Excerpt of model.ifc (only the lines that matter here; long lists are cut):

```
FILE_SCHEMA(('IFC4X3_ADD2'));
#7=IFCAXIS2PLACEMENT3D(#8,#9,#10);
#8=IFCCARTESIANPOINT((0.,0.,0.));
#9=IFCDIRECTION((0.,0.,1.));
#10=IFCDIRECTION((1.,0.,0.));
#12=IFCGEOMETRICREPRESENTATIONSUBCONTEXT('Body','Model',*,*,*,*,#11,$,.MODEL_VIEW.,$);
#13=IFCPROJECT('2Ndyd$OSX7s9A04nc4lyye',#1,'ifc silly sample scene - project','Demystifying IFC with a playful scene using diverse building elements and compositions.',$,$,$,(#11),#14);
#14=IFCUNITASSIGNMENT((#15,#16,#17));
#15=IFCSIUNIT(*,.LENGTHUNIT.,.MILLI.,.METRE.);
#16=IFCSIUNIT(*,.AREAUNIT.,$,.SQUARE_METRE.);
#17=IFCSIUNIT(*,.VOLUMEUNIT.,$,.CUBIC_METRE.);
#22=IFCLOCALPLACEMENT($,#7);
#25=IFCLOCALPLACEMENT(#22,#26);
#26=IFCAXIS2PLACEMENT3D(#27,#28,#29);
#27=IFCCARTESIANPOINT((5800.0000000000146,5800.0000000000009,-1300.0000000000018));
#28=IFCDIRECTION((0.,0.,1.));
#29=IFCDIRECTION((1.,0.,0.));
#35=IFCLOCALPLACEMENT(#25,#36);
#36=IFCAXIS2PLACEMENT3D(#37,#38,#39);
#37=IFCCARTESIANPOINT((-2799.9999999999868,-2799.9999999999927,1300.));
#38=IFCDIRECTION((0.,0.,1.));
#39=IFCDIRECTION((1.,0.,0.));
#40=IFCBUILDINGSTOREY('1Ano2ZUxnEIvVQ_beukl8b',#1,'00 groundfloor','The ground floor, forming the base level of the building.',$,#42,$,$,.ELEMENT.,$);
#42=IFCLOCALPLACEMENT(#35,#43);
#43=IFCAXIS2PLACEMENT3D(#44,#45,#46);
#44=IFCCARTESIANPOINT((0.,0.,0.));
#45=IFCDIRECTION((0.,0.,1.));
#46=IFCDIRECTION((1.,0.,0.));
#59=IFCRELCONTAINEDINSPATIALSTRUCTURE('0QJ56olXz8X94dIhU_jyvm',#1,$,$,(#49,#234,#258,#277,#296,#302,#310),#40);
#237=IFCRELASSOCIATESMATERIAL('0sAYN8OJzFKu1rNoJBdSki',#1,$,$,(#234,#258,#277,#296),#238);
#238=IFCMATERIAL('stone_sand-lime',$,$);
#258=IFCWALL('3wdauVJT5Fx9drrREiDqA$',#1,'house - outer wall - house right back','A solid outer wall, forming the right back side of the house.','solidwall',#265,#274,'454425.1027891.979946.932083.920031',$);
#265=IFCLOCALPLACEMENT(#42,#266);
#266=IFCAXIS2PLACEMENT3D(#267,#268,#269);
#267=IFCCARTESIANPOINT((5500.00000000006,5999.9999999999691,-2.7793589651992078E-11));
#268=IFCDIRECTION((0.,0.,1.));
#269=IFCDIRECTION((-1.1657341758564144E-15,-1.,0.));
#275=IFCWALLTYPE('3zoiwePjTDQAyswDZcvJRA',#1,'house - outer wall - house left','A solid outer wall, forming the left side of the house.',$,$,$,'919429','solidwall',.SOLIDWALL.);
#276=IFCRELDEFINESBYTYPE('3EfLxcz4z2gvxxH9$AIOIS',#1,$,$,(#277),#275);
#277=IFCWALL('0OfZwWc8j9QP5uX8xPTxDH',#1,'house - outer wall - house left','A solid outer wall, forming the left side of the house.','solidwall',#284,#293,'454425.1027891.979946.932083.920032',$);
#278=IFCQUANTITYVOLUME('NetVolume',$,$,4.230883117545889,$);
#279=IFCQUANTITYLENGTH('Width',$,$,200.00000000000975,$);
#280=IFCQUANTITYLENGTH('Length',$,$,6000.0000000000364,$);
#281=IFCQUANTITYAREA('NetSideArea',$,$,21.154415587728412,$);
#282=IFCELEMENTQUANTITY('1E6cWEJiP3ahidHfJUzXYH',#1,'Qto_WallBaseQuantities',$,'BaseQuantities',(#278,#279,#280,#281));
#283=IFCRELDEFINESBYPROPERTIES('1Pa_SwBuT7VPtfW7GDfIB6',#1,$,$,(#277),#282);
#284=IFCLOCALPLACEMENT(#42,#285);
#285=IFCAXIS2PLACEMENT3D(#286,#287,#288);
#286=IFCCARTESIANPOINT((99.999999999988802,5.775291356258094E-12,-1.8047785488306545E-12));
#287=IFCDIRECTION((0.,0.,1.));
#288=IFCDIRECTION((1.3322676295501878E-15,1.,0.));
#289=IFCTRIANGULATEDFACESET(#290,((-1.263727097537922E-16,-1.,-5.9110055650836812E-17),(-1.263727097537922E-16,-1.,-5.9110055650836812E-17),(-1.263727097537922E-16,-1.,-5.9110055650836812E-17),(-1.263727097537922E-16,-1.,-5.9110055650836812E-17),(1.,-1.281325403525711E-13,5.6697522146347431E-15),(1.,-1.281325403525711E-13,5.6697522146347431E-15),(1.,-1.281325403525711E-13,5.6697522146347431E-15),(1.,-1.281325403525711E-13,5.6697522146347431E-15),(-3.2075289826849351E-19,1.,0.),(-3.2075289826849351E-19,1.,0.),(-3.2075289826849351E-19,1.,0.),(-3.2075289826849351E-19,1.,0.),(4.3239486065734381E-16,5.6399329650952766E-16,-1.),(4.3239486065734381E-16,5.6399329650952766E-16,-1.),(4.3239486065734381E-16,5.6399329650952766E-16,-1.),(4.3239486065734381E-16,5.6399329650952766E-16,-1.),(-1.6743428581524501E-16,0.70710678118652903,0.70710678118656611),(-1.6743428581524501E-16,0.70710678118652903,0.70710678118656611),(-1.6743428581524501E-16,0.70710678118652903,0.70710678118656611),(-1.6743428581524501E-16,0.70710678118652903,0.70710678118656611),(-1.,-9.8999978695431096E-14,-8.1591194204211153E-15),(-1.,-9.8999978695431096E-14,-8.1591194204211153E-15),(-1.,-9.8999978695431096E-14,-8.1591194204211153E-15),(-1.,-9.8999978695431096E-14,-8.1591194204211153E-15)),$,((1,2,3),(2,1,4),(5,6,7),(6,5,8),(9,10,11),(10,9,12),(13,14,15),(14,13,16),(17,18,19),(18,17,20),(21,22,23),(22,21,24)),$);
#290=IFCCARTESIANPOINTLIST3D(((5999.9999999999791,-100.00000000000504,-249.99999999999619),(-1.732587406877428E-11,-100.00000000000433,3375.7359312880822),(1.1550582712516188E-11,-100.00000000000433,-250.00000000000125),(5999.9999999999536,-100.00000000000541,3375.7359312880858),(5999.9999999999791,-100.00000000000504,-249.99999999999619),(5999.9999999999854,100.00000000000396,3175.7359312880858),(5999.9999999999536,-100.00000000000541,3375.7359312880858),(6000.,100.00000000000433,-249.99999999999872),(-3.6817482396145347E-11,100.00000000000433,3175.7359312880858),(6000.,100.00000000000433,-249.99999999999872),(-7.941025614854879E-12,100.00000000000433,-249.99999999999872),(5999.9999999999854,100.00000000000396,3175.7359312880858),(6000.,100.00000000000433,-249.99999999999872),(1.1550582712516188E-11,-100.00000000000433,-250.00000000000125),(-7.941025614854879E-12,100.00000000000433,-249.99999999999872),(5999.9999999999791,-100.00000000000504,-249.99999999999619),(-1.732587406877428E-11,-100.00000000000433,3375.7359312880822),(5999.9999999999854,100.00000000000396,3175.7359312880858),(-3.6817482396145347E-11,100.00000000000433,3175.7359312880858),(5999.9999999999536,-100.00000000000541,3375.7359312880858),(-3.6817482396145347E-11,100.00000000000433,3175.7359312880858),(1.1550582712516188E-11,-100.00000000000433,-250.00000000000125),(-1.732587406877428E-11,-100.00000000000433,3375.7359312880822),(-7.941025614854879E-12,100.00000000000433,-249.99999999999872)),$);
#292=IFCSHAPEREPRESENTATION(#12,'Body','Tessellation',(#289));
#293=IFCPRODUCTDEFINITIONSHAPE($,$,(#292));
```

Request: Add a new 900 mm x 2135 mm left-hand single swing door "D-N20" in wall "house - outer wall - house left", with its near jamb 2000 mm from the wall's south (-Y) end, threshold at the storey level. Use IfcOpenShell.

```python
import numpy as np
import ifcopenshell
import ifcopenshell.api.feature
import ifcopenshell.api.geometry
import ifcopenshell.api.pset
import ifcopenshell.api.root
import ifcopenshell.api.spatial
import ifcopenshell.geom
import ifcopenshell.util.element
import ifcopenshell.util.placement
import ifcopenshell.util.representation
import ifcopenshell.util.shape
import ifcopenshell.util.unit

model = ifcopenshell.open("model.ifc")
unit_scale = ifcopenshell.util.unit.calculate_unit_scale(model)
area_scale = ifcopenshell.util.unit.calculate_unit_scale(model, "AREAUNIT")
volume_scale = ifcopenshell.util.unit.calculate_unit_scale(model, "VOLUMEUNIT")
settings = ifcopenshell.geom.settings()


def volume(element):
    """Net volume in cubic metres, openings subtracted."""
    shape = ifcopenshell.geom.create_shape(settings, element)
    return ifcopenshell.util.shape.get_volume(shape.geometry)


wall = model.by_id(277)
storey = ifcopenshell.util.element.get_container(wall, ifc_class="IfcBuildingStorey")
context = ifcopenshell.util.representation.get_context(model, "Model", "Body", "MODEL_VIEW")
before = volume(wall)

width, height, from_end, sill = 0.9, 2.135, 2, 0.0  # metres

# The wall runs along its own X axis, and the end named is its -X end.
wall_shape = ifcopenshell.geom.create_shape(settings, wall)
x, y, z = ifcopenshell.util.shape.get_vertices(wall_shape.geometry).T
start = x.min() + from_end
face, thickness = float(y.min()), float(y.max() - y.min())
wall_matrix = ifcopenshell.util.placement.get_local_placement(wall.ObjectPlacement)
level = ifcopenshell.util.placement.get_local_placement(storey.ObjectPlacement)[2, 3]


def in_wall(x, y):
    """Placement at x, y metres in the wall's axes, at sill height."""
    matrix = wall_matrix.copy()
    matrix[:, 3] = wall_matrix @ np.array([x / unit_scale, y / unit_scale, 0.0, 1.0])
    matrix[2, 3] = level + sill / unit_scale
    return matrix


# Opening: a box that overshoots both wall faces by 50 mm.
opening = ifcopenshell.api.root.create_entity(model, ifc_class="IfcOpeningElement", predefined_type="OPENING")
box = ifcopenshell.api.geometry.add_wall_representation(
    model, context=context, length=width, height=height, thickness=thickness + 0.1
)
ifcopenshell.api.geometry.assign_representation(model, product=opening, representation=box)
ifcopenshell.api.geometry.edit_object_placement(model, product=opening, matrix=in_wall(start, face - 0.05), is_si=False)
ifcopenshell.api.feature.add_feature(model, feature=opening, element=wall)

door = ifcopenshell.api.root.create_entity(model, ifc_class="IfcDoor", name="D-N20", predefined_type="DOOR")
door.OverallWidth, door.OverallHeight = width / unit_scale, height / unit_scale
door.OperationType = "SINGLE_SWING_LEFT"
body = ifcopenshell.api.geometry.add_door_representation(
    model,
    context=context,
    overall_width=door.OverallWidth,
    overall_height=door.OverallHeight,
    operation_type="SINGLE_SWING_LEFT",
    lining_properties={"LiningDepth": thickness / unit_scale, "ThresholdDepth": thickness / unit_scale},
)
ifcopenshell.api.geometry.assign_representation(model, product=door, representation=body)
ifcopenshell.api.spatial.assign_container(model, products=[door], relating_structure=storey)
ifcopenshell.api.feature.add_filling(model, opening=opening, element=door)

# The lining spans the wall, so the door starts at the wall face.
ifcopenshell.api.geometry.edit_object_placement(model, product=door, matrix=in_wall(start, face), is_si=False)

after = volume(wall)

# Update the wall's stored quantities.
qto = model.by_id(ifcopenshell.util.element.get_pset(wall, "Qto_WallBaseQuantities", should_inherit=False)["id"])
ifcopenshell.api.pset.edit_qto(model, qto=qto, properties={
    "NetVolume": after / volume_scale,
    "NetSideArea": after / thickness / area_scale,
})

print(f"wall volume {before:.3f} -> {after:.3f} m3")

model.write("model_edited.ifc")
```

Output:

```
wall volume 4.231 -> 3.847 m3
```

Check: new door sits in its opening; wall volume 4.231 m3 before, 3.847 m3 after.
